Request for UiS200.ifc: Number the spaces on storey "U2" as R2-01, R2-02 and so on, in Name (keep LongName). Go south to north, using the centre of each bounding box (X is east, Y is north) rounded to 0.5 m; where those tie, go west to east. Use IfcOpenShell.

First a look at what the model holds.

```python
import ifcopenshell
import ifcopenshell.util.element
import ifcopenshell.util.placement

model = ifcopenshell.open("UiS200.ifc")
print(model.schema)
storey = next(s for s in model.by_type("IfcBuildingStorey") if s.Name == "U2")
spaces = [e for e in ifcopenshell.util.element.get_decomposition(storey) if e.is_a("IfcSpace")]
for e in sorted(spaces, key=lambda e: e.id()):
    origin = ifcopenshell.util.placement.get_local_placement(e.ObjectPlacement)[:3, 3]
    print(e.id(), e.Name, e.LongName, origin.round(2) + 0.0, sep=" | ")
```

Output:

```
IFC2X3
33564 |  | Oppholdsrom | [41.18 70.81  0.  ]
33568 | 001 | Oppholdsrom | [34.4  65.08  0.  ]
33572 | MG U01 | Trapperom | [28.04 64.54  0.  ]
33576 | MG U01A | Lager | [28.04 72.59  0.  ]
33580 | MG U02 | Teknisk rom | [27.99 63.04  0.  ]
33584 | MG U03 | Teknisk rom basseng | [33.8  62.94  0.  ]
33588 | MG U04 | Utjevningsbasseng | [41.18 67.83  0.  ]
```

```python
import ifcopenshell
import ifcopenshell.geom
import ifcopenshell.util.element
import ifcopenshell.util.shape

model = ifcopenshell.open("UiS200.ifc")
settings = ifcopenshell.geom.settings()
settings.set("use-world-coords", True)


def centre(element):
    shape = ifcopenshell.geom.create_shape(settings, element)
    return ifcopenshell.util.shape.get_bbox_centroid(shape.geometry)


storey = next(s for s in model.by_type("IfcBuildingStorey") if s.Name == "U2")
spaces = [e for e in ifcopenshell.util.element.get_decomposition(storey) if e.is_a("IfcSpace")]

# Insertion points can sit at a corner or the storey origin, so sort by the geometry (in metres).
centres = {e: centre(e) for e in spaces}
spaces.sort(key=lambda e: (round(centres[e][1] / 0.5), centres[e][0]))

for i, e in enumerate(spaces, start=1):
    number = f"R2-{i:02d}"
    e.Name = number
    print(e.id(), number)

model.write("UiS200_v2.ifc")
```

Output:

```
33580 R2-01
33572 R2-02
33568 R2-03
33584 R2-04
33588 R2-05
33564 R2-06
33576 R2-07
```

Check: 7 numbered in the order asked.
